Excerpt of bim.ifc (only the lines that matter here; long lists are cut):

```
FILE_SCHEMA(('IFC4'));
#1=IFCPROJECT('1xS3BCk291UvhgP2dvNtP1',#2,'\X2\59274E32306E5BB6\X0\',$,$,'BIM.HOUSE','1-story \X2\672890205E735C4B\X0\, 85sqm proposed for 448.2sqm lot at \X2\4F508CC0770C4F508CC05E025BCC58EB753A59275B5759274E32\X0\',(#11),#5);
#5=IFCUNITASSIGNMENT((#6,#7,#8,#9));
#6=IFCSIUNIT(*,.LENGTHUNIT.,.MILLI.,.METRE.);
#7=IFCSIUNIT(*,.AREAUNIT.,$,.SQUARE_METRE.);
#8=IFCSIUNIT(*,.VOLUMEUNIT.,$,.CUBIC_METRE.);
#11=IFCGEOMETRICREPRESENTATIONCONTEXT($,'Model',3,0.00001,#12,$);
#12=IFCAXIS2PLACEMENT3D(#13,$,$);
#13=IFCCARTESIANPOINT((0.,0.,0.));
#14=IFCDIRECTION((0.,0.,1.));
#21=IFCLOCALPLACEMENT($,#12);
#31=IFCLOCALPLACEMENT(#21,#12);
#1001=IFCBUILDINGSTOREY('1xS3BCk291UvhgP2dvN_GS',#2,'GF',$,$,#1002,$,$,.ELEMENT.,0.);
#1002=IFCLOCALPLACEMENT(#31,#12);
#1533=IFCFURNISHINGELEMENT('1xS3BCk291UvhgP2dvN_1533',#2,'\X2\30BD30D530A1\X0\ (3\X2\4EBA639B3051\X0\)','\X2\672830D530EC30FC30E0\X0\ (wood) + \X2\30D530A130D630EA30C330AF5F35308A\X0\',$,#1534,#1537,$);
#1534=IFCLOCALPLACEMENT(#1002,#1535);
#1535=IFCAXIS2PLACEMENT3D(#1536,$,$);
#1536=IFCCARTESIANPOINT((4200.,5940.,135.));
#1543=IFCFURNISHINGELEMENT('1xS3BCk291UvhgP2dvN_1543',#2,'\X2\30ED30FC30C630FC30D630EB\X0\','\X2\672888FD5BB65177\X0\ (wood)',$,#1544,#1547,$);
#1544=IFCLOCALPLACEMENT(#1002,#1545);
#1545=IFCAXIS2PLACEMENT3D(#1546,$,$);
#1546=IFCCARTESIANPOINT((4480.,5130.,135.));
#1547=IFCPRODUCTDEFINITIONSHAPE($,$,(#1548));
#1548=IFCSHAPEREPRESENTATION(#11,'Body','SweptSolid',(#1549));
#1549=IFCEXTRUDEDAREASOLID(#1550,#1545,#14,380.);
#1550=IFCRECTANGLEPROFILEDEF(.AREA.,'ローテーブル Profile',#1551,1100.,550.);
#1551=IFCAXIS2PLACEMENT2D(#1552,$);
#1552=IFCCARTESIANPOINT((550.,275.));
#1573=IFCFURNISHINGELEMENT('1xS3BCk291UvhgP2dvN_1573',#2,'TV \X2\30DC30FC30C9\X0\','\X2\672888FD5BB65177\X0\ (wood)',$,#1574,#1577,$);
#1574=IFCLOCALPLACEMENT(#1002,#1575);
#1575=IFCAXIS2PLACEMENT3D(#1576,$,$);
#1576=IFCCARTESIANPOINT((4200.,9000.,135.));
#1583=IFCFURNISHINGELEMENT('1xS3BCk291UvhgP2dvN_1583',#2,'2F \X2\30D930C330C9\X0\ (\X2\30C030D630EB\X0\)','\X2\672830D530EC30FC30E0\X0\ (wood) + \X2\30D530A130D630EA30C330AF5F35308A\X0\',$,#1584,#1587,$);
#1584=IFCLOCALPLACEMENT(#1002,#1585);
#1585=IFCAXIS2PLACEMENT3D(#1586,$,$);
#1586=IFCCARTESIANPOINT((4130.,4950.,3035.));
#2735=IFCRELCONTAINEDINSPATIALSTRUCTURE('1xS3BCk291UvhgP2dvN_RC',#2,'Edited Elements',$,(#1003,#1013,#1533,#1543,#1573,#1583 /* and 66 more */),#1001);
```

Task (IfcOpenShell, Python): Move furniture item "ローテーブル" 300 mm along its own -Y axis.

```python
import ifcopenshell
import ifcopenshell.api.geometry
import ifcopenshell.util.placement
import ifcopenshell.util.unit

model = ifcopenshell.open("bim.ifc")
unit_scale = ifcopenshell.util.unit.calculate_unit_scale(model)

item = model.by_guid("1xS3BCk291UvhgP2dvN_1543")
matrix = ifcopenshell.util.placement.get_local_placement(item.ObjectPlacement)
matrix[:3, 3] -= matrix[:3, 1] * 0.3 / unit_scale
ifcopenshell.api.geometry.edit_object_placement(model, product=item, matrix=matrix, is_si=False)

print(ifcopenshell.util.placement.get_local_placement(item.ObjectPlacement).round(3) + 0.0)

model.write("bim_rev.ifc")
```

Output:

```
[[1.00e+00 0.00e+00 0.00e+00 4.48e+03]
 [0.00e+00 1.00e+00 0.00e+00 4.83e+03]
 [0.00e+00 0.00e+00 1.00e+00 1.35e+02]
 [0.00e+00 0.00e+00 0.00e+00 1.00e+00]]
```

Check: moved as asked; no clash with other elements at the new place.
